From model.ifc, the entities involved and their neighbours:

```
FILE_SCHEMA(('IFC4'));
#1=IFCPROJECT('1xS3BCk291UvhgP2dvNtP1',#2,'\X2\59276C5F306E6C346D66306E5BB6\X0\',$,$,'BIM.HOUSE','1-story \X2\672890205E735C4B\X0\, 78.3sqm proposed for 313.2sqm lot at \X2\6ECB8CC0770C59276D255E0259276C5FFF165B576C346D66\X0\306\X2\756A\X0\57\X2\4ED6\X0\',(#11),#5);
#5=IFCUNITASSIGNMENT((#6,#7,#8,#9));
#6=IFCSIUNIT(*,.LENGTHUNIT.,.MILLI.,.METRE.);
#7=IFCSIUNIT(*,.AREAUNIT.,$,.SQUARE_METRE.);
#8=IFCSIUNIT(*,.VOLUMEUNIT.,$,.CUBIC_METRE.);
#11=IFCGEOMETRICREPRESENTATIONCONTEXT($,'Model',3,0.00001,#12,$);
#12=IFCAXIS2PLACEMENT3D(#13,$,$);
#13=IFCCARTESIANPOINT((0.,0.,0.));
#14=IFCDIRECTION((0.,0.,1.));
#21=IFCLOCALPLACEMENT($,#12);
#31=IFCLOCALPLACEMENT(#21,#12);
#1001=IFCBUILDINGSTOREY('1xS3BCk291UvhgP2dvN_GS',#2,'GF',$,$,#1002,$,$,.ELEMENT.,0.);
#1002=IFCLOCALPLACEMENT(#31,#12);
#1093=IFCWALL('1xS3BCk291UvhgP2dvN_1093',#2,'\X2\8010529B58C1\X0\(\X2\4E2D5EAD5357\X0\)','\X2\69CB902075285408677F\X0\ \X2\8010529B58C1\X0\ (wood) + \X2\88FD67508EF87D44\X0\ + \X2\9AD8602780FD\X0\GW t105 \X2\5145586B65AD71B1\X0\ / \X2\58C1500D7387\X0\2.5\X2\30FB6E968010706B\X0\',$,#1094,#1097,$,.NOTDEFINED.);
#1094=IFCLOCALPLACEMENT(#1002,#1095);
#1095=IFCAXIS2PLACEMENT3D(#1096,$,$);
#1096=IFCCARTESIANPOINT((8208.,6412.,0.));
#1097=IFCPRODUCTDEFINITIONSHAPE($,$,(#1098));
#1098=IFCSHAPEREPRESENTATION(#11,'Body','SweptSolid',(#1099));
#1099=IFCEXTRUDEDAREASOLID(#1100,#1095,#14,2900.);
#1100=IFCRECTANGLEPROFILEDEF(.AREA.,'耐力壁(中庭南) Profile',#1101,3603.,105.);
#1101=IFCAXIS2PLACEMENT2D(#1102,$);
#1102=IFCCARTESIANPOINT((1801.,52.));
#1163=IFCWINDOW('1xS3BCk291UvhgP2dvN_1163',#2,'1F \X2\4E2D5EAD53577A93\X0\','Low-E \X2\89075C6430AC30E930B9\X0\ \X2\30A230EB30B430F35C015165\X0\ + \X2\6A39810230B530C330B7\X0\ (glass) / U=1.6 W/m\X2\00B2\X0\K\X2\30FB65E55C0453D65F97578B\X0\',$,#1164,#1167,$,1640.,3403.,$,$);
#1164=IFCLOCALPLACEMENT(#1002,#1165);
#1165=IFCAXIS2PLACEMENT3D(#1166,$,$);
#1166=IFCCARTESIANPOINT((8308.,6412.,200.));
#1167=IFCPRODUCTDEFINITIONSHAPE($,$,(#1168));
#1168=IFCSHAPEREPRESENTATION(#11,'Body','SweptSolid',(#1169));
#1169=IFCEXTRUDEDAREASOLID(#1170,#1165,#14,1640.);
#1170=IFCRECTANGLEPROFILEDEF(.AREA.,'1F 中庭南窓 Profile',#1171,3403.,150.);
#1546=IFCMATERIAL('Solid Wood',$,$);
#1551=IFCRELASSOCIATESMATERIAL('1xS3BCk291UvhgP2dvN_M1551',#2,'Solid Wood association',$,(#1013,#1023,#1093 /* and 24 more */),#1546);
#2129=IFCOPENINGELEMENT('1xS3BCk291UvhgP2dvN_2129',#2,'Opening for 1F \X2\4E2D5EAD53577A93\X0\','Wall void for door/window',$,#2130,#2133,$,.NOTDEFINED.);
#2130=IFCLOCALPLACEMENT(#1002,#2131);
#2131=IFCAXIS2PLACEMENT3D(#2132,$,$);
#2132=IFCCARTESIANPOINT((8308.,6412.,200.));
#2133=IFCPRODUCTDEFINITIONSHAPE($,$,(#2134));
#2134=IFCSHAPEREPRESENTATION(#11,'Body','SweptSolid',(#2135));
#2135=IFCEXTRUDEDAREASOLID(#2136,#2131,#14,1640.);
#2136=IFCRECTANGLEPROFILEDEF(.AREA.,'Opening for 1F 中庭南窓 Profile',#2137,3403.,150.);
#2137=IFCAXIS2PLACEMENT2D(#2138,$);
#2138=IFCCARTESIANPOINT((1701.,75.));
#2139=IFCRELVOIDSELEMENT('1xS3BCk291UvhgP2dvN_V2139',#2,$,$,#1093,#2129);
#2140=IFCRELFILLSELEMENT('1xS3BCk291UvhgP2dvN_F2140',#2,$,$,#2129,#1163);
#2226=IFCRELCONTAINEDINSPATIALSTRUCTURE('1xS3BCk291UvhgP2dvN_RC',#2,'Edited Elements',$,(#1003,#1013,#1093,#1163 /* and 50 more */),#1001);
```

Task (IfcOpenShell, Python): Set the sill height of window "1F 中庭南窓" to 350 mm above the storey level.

```python
import numpy as np
import ifcopenshell
import ifcopenshell.api.geometry
import ifcopenshell.geom
import ifcopenshell.util.element
import ifcopenshell.util.placement
import ifcopenshell.util.shape
import ifcopenshell.util.unit

model = ifcopenshell.open("model.ifc")
unit_scale = ifcopenshell.util.unit.calculate_unit_scale(model)

window = model.by_id(1163)
opening = window.FillsVoids[0].RelatingOpeningElement
storey = ifcopenshell.util.element.get_container(window, ifc_class="IfcBuildingStorey")
level = ifcopenshell.util.placement.get_local_placement(storey.ObjectPlacement)[2, 3]

# The opening's origin need not be at the sill, so measure its lowest point.
shape = ifcopenshell.geom.create_shape(ifcopenshell.geom.settings(), opening)
bottom = ifcopenshell.util.shape.get_shape_bottom_elevation(shape, shape.geometry) / unit_scale
dz = level + 350.0 - bottom

shift = np.array([0.0, 0.0, dz])
# The window is not placed relative to its opening, so move both.
for product in (opening, window):
    matrix = ifcopenshell.util.placement.get_local_placement(product.ObjectPlacement)
    matrix[:3, 3] += shift
    ifcopenshell.api.geometry.edit_object_placement(model, product=product, matrix=matrix, is_si=False)

print(f"moved by {dz * unit_scale:+.3f} m")

model.write("model_rev.ifc")
```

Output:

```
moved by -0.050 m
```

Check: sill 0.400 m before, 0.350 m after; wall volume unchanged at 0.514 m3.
